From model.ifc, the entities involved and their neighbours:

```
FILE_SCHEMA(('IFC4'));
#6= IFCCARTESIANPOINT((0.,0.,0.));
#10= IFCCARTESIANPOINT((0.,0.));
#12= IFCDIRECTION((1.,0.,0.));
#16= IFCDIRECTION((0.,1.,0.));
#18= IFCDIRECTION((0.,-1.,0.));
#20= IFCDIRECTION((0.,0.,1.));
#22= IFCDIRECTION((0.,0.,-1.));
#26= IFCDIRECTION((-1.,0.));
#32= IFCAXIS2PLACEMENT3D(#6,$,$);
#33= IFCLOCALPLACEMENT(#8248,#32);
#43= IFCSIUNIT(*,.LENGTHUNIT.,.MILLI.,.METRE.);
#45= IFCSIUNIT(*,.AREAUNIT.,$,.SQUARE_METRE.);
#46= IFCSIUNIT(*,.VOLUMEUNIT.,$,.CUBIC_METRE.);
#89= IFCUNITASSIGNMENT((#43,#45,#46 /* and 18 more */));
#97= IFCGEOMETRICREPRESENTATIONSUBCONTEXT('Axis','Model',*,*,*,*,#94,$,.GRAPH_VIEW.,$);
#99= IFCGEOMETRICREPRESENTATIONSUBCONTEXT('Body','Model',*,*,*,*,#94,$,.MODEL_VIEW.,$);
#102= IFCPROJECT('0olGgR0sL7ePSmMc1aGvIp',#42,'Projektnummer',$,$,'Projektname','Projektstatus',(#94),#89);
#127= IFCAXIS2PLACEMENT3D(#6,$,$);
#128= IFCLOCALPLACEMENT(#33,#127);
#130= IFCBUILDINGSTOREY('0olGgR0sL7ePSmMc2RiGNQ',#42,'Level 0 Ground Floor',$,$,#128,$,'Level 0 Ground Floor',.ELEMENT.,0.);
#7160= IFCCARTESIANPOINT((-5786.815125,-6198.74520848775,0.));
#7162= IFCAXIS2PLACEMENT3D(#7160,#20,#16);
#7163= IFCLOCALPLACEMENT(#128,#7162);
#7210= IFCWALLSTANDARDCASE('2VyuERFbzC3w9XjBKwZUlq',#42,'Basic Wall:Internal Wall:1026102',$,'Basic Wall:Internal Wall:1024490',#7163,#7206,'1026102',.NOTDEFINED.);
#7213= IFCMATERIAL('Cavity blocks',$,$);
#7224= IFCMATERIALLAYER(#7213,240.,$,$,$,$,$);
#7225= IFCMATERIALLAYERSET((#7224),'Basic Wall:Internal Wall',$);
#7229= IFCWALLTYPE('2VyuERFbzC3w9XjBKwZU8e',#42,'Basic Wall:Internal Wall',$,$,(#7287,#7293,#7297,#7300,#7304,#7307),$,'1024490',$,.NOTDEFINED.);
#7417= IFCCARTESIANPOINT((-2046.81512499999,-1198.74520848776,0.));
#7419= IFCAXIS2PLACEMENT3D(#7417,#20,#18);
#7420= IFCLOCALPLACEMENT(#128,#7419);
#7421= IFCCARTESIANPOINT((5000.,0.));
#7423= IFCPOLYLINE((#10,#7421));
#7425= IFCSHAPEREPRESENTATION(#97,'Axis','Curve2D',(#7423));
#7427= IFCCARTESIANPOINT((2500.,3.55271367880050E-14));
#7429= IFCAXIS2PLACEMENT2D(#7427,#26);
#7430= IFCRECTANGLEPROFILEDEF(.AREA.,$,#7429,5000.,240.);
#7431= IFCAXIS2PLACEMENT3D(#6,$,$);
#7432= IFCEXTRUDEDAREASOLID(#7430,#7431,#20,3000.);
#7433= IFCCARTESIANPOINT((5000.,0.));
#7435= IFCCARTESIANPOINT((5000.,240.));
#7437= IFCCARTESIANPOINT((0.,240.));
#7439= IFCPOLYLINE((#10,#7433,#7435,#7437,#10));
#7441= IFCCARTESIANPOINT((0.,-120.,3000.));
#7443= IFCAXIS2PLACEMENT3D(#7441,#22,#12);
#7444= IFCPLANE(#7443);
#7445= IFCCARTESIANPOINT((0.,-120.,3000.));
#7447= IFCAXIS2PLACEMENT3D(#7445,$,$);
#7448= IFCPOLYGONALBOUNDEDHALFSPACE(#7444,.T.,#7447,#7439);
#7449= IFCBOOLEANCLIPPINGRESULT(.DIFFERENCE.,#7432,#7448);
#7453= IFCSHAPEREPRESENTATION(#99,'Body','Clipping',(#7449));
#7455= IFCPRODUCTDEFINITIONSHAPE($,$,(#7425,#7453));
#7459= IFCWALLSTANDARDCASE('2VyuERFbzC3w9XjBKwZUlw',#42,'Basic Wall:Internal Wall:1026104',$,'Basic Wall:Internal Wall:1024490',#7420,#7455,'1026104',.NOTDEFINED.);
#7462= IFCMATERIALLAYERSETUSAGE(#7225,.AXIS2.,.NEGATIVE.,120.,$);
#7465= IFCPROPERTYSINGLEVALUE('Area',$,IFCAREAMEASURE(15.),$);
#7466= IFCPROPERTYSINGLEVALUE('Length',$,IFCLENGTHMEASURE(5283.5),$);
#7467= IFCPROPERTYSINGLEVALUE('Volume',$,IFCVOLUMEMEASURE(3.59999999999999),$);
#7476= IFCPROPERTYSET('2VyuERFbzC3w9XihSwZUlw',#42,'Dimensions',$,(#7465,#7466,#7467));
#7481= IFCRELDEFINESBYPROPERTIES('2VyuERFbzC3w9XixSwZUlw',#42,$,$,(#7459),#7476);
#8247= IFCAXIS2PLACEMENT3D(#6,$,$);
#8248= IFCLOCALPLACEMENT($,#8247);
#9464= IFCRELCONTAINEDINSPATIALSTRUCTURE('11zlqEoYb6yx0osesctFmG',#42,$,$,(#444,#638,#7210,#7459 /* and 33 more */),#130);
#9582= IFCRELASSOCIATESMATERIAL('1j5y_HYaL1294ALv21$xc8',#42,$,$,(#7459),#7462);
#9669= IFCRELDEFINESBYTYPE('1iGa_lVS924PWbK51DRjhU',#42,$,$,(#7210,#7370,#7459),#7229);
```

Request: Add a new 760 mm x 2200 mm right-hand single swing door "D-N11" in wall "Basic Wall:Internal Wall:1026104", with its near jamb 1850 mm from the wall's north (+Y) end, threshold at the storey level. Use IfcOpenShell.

```python
import numpy as np
import ifcopenshell
import ifcopenshell.api.feature
import ifcopenshell.api.geometry
import ifcopenshell.api.pset
import ifcopenshell.api.root
import ifcopenshell.api.spatial
import ifcopenshell.geom
import ifcopenshell.util.element
import ifcopenshell.util.placement
import ifcopenshell.util.representation
import ifcopenshell.util.shape
import ifcopenshell.util.unit

model = ifcopenshell.open("model.ifc")
unit_scale = ifcopenshell.util.unit.calculate_unit_scale(model)
area_scale = ifcopenshell.util.unit.calculate_unit_scale(model, "AREAUNIT")
volume_scale = ifcopenshell.util.unit.calculate_unit_scale(model, "VOLUMEUNIT")
settings = ifcopenshell.geom.settings()


def volume(element):
    """Net volume in cubic metres, openings subtracted."""
    shape = ifcopenshell.geom.create_shape(settings, element)
    return ifcopenshell.util.shape.get_volume(shape.geometry)


wall = model.by_id(7459)
storey = ifcopenshell.util.element.get_container(wall, ifc_class="IfcBuildingStorey")
context = ifcopenshell.util.representation.get_context(model, "Model", "Body", "MODEL_VIEW")
before = volume(wall)

width, height, from_end, sill = 0.76, 2.2, 1.85, 0.0  # metres

# The wall runs along its own X axis, and the end named is its -X end.
wall_shape = ifcopenshell.geom.create_shape(settings, wall)
x, y, z = ifcopenshell.util.shape.get_vertices(wall_shape.geometry).T
start = x.min() + from_end
face, thickness = float(y.min()), float(y.max() - y.min())
wall_matrix = ifcopenshell.util.placement.get_local_placement(wall.ObjectPlacement)
level = ifcopenshell.util.placement.get_local_placement(storey.ObjectPlacement)[2, 3]


def in_wall(x, y):
    """Placement at x, y metres in the wall's axes, at sill height."""
    matrix = wall_matrix.copy()
    matrix[:, 3] = wall_matrix @ np.array([x / unit_scale, y / unit_scale, 0.0, 1.0])
    matrix[2, 3] = level + sill / unit_scale
    return matrix


# Opening: a box that overshoots both wall faces by 50 mm.
opening = ifcopenshell.api.root.create_entity(model, ifc_class="IfcOpeningElement", predefined_type="OPENING")
box = ifcopenshell.api.geometry.add_wall_representation(
    model, context=context, length=width, height=height, thickness=thickness + 0.1
)
ifcopenshell.api.geometry.assign_representation(model, product=opening, representation=box)
ifcopenshell.api.geometry.edit_object_placement(model, product=opening, matrix=in_wall(start, face - 0.05), is_si=False)
ifcopenshell.api.feature.add_feature(model, feature=opening, element=wall)

door = ifcopenshell.api.root.create_entity(model, ifc_class="IfcDoor", name="D-N11", predefined_type="DOOR")
door.OverallWidth, door.OverallHeight = width / unit_scale, height / unit_scale
door.OperationType = "SINGLE_SWING_RIGHT"
body = ifcopenshell.api.geometry.add_door_representation(
    model,
    context=context,
    overall_width=door.OverallWidth,
    overall_height=door.OverallHeight,
    operation_type="SINGLE_SWING_RIGHT",
    lining_properties={"LiningDepth": thickness / unit_scale, "ThresholdDepth": thickness / unit_scale},
)
ifcopenshell.api.geometry.assign_representation(model, product=door, representation=body)
ifcopenshell.api.spatial.assign_container(model, products=[door], relating_structure=storey)
ifcopenshell.api.feature.add_filling(model, opening=opening, element=door)

# The lining spans the wall, so the door starts at the wall face.
ifcopenshell.api.geometry.edit_object_placement(model, product=door, matrix=in_wall(start, face), is_si=False)

after = volume(wall)

# Update the wall's stored quantities.
pset = model.by_id(ifcopenshell.util.element.get_pset(wall, "Dimensions", should_inherit=False)["id"])
ifcopenshell.api.pset.edit_pset(model, pset=pset, properties={
    "Area": model.create_entity("IfcAreaMeasure", after / thickness / area_scale),
    "Volume": model.create_entity("IfcVolumeMeasure", after / volume_scale),
})

print(f"wall volume {before:.3f} -> {after:.3f} m3")

model.write("model_edited.ifc")
```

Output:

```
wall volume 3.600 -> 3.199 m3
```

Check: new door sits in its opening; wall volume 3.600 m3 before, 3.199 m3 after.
